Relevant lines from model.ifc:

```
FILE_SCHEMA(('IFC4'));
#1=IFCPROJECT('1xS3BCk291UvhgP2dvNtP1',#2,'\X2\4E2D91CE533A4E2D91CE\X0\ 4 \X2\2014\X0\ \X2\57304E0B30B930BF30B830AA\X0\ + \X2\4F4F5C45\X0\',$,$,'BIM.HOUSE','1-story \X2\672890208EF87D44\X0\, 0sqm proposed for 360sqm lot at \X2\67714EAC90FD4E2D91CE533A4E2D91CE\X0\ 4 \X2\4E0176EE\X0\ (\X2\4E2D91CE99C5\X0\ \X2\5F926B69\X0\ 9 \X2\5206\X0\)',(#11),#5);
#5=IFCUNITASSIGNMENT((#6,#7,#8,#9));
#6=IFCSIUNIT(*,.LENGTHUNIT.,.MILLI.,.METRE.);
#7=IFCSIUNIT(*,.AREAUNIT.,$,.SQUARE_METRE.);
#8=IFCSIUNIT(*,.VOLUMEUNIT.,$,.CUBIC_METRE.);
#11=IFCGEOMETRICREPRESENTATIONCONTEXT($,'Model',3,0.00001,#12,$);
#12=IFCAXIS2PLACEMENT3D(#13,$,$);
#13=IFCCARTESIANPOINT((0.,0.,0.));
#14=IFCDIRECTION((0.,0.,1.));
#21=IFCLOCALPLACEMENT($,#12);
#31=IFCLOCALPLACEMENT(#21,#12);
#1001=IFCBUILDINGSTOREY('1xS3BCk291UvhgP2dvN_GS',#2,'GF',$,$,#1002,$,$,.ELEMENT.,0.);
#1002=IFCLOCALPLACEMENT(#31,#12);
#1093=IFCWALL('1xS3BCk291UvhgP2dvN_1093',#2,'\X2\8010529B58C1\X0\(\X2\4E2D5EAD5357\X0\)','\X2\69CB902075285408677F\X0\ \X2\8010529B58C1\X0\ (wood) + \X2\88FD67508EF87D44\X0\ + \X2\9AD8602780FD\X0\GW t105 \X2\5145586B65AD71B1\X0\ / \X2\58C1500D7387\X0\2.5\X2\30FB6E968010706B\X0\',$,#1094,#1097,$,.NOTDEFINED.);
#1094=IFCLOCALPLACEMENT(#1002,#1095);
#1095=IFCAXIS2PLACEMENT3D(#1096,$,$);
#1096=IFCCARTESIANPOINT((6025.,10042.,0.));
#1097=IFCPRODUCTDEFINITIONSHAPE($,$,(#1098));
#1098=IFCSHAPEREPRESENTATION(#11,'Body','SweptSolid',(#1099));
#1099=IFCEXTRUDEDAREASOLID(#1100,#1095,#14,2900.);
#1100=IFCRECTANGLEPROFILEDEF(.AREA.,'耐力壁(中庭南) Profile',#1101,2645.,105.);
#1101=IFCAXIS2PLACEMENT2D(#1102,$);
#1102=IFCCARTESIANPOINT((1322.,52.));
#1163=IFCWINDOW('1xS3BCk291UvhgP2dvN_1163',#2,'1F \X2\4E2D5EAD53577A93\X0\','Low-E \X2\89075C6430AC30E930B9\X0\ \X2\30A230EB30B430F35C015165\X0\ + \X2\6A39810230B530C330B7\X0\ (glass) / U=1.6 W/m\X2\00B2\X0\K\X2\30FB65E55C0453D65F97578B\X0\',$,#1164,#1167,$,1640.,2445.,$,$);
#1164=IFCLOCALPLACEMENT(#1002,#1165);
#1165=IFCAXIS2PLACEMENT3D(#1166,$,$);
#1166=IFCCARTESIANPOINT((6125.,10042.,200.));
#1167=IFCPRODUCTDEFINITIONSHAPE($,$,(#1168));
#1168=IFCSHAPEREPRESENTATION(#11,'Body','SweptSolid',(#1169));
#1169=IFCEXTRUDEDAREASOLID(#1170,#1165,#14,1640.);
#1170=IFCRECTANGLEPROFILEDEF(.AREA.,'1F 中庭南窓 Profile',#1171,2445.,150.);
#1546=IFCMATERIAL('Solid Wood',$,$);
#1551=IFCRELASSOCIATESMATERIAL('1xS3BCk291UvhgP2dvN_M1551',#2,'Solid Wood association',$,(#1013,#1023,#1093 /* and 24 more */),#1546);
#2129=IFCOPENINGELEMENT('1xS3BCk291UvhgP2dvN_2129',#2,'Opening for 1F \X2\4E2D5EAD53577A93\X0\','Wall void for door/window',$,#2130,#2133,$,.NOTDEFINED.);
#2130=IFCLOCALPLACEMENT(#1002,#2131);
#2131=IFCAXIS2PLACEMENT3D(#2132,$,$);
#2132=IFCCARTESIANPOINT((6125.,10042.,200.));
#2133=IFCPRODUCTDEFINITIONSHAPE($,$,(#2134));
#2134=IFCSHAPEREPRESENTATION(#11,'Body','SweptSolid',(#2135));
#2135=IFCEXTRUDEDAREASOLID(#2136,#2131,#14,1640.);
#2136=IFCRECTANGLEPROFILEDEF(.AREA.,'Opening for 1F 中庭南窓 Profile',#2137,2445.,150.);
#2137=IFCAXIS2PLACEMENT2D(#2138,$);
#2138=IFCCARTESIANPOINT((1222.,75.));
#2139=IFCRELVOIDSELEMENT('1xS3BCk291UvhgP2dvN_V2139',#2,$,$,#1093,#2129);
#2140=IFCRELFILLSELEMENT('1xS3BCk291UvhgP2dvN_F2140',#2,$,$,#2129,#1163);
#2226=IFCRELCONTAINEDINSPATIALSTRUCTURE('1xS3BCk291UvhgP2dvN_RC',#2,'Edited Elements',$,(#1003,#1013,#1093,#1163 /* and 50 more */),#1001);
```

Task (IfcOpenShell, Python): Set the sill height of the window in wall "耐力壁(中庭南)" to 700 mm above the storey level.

```python
import numpy as np
import ifcopenshell
import ifcopenshell.api.geometry
import ifcopenshell.geom
import ifcopenshell.util.element
import ifcopenshell.util.placement
import ifcopenshell.util.shape
import ifcopenshell.util.unit

model = ifcopenshell.open("model.ifc")
unit_scale = ifcopenshell.util.unit.calculate_unit_scale(model)

window = model.by_guid("1xS3BCk291UvhgP2dvN_1163")
opening = window.FillsVoids[0].RelatingOpeningElement
storey = ifcopenshell.util.element.get_container(window, ifc_class="IfcBuildingStorey")
level = ifcopenshell.util.placement.get_local_placement(storey.ObjectPlacement)[2, 3]

# The opening's origin need not be at the sill, so measure its lowest point.
shape = ifcopenshell.geom.create_shape(ifcopenshell.geom.settings(), opening)
bottom = ifcopenshell.util.shape.get_shape_bottom_elevation(shape, shape.geometry) / unit_scale
dz = level + 700.0 - bottom

shift = np.array([0.0, 0.0, dz])
# The window is not placed relative to its opening, so move both.
for product in (opening, window):
    matrix = ifcopenshell.util.placement.get_local_placement(product.ObjectPlacement)
    matrix[:3, 3] += shift
    ifcopenshell.api.geometry.edit_object_placement(model, product=product, matrix=matrix, is_si=False)

print(f"moved by {dz * unit_scale:+.3f} m")

model.write("model_v2.ifc")
```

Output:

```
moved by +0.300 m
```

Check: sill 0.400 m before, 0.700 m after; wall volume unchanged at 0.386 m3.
